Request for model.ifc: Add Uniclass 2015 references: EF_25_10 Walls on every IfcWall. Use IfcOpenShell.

First a look at what the model holds.

```python
import ifcopenshell

model = ifcopenshell.open("model.ifc")
print(model.schema)
print("classifications:", [c.Name for c in model.by_type("IfcClassification")])
for ifc_class in ("IfcDoor", "IfcRoof", "IfcStair", "IfcWall", "IfcWindow"):
    print(ifc_class, len(model.by_type(ifc_class)))
```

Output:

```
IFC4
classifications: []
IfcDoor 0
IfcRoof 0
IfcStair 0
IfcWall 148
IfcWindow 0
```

```python
import ifcopenshell
import ifcopenshell.api.classification

model = ifcopenshell.open("model.ifc")

system = ifcopenshell.api.classification.add_classification(model, classification="Uniclass 2015")

codes = {
    "IfcWall": ("EF_25_10", "Walls"),
}
for ifc_class, (code, name) in codes.items():
    products = model.by_type(ifc_class)
    ifcopenshell.api.classification.add_reference(
        model, products=products, classification=system, identification=code, name=name
    )
    print(code, len(products))

model.write("model_edited.ifc")
```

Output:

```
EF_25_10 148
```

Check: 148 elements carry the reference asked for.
